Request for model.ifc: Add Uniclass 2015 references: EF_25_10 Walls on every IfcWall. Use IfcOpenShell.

First a look at what the model holds.

```python
import ifcopenshell

model = ifcopenshell.open("model.ifc")
print(model.schema)
print("classifications:", [c.Name for c in model.by_type("IfcClassification")])
for ifc_class in ("IfcDoor", "IfcRoof", "IfcStair", "IfcWall", "IfcWindow"):
    print(ifc_class, len(model.by_type(ifc_class)))
```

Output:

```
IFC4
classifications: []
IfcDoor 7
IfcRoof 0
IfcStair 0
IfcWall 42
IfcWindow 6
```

```python
import ifcopenshell
import ifcopenshell.api.classification

model = ifcopenshell.open("model.ifc")

system = ifcopenshell.api.classification.add_classification(model, classification="Uniclass 2015")

codes = {
    "IfcWall": ("EF_25_10", "Walls"),
}
for ifc_class, (code, name) in codes.items():
    products = model.by_type(ifc_class)
    ifcopenshell.api.classification.add_reference(
        model, products=products, classification=system, identification=code, name=name
    )
    print(code, len(products))

model.write("model-out.ifc")
```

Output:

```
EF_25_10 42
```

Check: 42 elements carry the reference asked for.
